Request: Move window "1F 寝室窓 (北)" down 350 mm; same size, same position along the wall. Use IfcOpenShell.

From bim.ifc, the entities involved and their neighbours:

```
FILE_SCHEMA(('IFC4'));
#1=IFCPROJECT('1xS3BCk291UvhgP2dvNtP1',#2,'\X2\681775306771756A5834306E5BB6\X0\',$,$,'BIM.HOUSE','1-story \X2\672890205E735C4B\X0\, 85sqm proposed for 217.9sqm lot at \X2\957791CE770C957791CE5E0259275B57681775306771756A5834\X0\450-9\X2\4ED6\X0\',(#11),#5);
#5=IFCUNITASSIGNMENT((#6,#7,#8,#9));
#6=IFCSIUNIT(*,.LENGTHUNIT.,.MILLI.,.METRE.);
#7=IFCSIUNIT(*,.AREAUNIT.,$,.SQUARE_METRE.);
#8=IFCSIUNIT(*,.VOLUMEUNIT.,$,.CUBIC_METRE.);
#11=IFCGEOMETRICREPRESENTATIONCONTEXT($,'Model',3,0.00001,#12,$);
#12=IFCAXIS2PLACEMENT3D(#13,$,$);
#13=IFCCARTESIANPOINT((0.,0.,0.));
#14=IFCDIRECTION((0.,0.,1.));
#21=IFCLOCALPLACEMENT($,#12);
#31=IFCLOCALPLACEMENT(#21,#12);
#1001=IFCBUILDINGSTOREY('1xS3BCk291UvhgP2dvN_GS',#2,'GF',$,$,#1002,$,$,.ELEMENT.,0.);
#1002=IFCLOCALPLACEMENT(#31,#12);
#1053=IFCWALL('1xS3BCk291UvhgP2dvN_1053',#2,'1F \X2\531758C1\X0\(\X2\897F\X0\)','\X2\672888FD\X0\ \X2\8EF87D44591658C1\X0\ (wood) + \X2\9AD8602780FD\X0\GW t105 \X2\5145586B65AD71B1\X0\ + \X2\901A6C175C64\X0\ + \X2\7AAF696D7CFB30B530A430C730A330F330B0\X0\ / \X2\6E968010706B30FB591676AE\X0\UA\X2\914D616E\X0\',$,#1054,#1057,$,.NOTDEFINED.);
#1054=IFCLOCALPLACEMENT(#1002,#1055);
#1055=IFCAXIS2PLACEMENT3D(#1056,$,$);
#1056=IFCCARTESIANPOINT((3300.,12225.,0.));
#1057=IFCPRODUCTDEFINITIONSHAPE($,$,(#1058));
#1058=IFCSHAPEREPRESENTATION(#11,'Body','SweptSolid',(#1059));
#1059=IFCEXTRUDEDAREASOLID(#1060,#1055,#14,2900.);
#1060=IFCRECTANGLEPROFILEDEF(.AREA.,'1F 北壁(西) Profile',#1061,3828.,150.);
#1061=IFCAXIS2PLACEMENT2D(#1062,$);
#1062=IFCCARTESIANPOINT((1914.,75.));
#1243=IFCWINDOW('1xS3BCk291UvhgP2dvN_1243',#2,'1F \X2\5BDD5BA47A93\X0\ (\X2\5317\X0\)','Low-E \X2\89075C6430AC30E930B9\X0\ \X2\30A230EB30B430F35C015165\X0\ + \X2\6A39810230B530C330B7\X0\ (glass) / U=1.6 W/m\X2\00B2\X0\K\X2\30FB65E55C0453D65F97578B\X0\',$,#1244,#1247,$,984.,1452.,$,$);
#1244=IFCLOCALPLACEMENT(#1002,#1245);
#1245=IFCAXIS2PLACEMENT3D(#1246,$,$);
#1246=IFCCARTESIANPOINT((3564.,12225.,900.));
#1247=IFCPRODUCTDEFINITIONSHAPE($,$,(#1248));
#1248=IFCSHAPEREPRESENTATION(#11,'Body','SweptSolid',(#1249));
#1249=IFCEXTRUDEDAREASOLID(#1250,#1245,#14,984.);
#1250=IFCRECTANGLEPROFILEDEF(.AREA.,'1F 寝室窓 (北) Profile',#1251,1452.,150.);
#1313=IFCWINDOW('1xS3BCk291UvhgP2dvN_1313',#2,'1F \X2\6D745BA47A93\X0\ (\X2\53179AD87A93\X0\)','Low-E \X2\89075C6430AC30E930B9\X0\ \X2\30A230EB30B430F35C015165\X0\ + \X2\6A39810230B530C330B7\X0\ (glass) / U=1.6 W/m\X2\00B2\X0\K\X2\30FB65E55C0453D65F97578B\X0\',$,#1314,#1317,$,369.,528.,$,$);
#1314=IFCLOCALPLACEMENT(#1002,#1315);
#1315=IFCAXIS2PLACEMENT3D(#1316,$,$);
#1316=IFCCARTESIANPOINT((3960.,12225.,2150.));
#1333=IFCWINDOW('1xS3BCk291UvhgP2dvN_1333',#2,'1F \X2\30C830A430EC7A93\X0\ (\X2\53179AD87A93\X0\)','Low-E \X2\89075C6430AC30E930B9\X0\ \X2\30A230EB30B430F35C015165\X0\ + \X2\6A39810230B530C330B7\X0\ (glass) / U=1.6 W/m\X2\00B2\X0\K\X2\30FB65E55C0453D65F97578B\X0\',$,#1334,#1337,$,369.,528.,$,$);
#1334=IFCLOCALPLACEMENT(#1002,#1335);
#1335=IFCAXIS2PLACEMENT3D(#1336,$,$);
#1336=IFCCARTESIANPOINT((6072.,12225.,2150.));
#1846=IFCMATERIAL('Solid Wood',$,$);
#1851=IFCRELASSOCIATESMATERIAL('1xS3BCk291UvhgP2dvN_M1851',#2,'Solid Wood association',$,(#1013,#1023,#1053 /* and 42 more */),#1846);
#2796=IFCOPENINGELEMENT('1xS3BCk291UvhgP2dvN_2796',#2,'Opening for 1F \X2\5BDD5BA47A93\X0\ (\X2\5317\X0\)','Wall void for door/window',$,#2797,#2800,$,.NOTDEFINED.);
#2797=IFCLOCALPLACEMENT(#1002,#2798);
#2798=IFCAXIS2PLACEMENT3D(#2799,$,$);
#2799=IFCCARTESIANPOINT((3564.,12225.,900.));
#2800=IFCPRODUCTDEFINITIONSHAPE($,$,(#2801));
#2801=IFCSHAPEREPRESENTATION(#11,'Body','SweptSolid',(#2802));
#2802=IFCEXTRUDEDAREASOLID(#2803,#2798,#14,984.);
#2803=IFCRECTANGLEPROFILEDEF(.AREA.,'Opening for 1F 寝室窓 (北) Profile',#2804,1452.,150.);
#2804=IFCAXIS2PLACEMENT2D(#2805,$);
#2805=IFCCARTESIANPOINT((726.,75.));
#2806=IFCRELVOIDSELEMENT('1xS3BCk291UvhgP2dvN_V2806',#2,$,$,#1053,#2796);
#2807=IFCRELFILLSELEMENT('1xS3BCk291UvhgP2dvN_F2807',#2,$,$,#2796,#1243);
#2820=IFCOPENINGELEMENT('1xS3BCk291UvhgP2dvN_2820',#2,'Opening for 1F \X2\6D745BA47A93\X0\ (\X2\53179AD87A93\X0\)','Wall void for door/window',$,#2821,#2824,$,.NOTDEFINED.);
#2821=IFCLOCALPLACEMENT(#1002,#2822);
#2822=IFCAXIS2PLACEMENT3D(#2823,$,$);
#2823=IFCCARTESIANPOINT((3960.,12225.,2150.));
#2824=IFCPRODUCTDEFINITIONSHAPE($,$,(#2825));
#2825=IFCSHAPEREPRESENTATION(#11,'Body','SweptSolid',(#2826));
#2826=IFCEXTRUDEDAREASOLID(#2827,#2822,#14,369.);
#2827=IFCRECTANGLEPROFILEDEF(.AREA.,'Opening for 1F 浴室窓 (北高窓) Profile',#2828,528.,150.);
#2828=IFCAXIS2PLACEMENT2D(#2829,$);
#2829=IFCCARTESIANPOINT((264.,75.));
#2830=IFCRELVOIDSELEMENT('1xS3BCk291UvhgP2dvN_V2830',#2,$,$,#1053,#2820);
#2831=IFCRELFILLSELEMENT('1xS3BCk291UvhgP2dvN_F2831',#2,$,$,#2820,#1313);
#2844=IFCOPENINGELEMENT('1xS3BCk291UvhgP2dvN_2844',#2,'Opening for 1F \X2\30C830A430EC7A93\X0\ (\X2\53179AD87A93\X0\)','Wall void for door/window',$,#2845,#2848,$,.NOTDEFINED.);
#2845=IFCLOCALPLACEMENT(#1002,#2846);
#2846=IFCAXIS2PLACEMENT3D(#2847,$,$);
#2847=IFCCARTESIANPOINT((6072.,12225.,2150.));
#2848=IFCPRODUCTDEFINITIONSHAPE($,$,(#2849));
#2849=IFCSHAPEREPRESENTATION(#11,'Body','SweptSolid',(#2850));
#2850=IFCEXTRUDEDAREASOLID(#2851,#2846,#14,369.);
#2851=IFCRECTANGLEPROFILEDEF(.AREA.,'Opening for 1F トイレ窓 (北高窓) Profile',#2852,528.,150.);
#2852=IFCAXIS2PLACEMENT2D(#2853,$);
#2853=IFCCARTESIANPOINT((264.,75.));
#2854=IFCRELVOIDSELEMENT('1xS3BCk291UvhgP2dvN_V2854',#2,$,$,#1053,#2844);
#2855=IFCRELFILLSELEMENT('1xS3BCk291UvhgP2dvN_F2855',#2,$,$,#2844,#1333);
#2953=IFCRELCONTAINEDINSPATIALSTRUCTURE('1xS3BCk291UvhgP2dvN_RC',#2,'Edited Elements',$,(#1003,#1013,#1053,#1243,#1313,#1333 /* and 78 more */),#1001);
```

```python
import numpy as np
import ifcopenshell
import ifcopenshell.api.geometry
import ifcopenshell.util.placement
import ifcopenshell.util.unit

model = ifcopenshell.open("bim.ifc")
unit_scale = ifcopenshell.util.unit.calculate_unit_scale(model)

window = model.by_guid("1xS3BCk291UvhgP2dvN_1243")
opening = window.FillsVoids[0].RelatingOpeningElement
dz = -0.35 / unit_scale

shift = np.array([0.0, 0.0, dz])
# The window is not placed relative to its opening, so move both.
for product in (opening, window):
    matrix = ifcopenshell.util.placement.get_local_placement(product.ObjectPlacement)
    matrix[:3, 3] += shift
    ifcopenshell.api.geometry.edit_object_placement(model, product=product, matrix=matrix, is_si=False)

print(f"moved by {dz * unit_scale:+.3f} m")

model.write("bim_rev.ifc")
```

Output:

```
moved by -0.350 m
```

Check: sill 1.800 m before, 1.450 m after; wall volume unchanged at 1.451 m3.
